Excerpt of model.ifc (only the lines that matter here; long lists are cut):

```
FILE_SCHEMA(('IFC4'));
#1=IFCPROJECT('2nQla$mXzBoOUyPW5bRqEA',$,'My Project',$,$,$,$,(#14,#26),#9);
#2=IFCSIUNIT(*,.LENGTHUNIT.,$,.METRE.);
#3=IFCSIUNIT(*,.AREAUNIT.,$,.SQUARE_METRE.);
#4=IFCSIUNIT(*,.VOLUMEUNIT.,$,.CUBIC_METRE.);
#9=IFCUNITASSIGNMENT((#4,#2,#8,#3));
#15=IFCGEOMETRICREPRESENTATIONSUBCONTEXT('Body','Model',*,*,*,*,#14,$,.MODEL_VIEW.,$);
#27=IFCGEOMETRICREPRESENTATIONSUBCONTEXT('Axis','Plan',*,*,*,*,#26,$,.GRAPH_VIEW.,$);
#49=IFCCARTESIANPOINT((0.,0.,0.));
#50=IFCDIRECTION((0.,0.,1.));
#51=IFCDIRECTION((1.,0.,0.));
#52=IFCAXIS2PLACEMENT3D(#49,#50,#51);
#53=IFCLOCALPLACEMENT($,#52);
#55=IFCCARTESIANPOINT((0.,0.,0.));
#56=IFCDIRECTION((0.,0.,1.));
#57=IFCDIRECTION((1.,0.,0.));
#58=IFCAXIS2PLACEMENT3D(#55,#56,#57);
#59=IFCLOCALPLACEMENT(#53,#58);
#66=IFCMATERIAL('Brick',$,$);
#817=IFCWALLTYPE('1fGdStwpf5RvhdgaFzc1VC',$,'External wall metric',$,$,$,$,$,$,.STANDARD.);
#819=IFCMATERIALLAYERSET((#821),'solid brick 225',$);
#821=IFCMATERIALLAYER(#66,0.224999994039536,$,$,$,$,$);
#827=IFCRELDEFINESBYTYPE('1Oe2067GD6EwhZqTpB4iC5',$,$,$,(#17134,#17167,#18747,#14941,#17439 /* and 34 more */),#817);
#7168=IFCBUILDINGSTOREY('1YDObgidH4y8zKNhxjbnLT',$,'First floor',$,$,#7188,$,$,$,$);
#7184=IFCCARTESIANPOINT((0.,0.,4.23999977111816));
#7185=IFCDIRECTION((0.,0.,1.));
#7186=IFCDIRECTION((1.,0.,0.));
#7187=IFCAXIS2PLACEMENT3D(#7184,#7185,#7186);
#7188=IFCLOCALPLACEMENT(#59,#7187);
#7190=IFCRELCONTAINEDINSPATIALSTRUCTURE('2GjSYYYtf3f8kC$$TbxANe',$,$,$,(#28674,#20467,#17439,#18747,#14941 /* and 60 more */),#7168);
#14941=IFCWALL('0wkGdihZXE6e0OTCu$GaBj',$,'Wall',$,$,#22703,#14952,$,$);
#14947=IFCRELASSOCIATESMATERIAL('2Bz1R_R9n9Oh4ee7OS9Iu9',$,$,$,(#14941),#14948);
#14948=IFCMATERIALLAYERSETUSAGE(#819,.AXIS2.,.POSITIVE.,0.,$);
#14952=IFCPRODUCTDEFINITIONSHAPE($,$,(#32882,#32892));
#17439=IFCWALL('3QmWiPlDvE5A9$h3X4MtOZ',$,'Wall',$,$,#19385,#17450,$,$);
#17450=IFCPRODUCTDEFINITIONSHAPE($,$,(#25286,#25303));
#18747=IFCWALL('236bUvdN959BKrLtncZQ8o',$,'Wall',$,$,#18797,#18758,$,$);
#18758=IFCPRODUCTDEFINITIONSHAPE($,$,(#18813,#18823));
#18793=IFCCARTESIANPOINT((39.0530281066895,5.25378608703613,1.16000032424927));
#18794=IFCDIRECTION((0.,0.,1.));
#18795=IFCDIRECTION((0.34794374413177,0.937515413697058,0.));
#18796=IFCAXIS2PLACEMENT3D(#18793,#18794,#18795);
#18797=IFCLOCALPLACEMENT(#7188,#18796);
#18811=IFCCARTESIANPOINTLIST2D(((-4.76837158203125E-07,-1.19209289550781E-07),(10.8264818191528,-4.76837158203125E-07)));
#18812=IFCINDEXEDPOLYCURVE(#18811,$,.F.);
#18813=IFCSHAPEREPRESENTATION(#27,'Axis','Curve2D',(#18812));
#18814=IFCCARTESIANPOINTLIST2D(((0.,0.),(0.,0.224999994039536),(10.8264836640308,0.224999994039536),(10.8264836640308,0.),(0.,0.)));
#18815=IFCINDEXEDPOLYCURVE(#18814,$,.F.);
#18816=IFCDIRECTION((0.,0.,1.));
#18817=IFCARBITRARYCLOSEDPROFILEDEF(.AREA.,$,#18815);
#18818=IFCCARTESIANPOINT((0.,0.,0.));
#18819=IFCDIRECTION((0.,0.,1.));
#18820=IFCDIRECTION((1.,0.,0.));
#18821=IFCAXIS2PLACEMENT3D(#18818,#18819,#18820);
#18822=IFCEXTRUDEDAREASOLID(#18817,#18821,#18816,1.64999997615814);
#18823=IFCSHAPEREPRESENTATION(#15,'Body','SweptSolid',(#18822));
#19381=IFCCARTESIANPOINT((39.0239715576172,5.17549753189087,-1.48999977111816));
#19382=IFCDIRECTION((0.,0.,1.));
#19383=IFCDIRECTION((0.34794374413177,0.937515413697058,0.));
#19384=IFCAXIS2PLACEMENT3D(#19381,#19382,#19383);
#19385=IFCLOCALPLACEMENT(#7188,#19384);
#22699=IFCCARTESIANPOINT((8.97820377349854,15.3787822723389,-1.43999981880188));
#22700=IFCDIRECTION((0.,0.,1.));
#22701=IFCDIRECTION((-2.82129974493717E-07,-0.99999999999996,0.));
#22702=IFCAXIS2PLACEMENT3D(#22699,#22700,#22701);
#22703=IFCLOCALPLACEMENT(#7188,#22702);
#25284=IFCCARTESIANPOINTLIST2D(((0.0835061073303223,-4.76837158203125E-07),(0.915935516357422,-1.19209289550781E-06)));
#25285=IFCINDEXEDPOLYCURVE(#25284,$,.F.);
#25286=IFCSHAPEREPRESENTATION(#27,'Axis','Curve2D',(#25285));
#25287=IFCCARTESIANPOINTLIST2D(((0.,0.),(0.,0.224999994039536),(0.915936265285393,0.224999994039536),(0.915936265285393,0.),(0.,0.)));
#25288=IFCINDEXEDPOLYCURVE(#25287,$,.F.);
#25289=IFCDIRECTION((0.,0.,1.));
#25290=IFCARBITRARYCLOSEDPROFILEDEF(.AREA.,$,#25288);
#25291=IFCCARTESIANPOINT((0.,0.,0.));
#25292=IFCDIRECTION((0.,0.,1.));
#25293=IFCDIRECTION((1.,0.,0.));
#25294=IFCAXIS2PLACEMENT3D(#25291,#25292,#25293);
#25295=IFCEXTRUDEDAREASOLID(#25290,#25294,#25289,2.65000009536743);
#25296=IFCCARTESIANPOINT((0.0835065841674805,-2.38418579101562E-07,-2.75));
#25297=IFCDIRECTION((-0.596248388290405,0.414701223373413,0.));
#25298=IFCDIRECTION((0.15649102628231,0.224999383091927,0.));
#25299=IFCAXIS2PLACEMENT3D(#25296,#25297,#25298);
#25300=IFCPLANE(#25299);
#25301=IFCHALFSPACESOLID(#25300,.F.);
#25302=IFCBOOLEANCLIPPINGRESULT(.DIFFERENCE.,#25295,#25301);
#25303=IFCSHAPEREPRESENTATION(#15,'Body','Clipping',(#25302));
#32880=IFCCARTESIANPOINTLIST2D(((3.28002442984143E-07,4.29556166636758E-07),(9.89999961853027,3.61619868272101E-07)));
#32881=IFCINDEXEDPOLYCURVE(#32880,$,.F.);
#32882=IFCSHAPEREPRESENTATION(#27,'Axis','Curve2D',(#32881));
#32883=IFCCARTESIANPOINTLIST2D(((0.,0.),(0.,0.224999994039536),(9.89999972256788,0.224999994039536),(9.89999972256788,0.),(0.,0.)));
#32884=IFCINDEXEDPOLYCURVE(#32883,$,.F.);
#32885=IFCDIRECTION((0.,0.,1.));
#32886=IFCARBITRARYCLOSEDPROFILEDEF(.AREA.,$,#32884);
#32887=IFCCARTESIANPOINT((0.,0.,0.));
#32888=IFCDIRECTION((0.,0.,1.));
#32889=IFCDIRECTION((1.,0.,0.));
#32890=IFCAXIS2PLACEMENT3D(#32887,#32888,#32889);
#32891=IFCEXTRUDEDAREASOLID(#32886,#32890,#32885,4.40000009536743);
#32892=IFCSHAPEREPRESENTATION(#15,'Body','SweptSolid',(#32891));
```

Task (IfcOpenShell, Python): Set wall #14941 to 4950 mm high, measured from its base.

```python
import ifcopenshell
import ifcopenshell.geom
import ifcopenshell.util.representation
import ifcopenshell.util.shape
import ifcopenshell.util.unit

model = ifcopenshell.open("model.ifc")
unit_scale = ifcopenshell.util.unit.calculate_unit_scale(model)
settings = ifcopenshell.geom.settings()


def volume(element):
    """Net volume in cubic metres, openings subtracted."""
    shape = ifcopenshell.geom.create_shape(settings, element)
    return ifcopenshell.util.shape.get_volume(shape.geometry)


wall = model.by_guid("0wkGdihZXE6e0OTCu$GaBj")
before = volume(wall)

body = ifcopenshell.util.representation.get_representation(wall, "Model", "Body")
solid = body.Items[0]
old_height = solid.Depth
solid.Depth = 4.95 / unit_scale
after = volume(wall)

print(f"height {old_height:g} -> {solid.Depth:g}, volume {before:.3f} -> {after:.3f} m3")

model.write("model_edited.ifc")
```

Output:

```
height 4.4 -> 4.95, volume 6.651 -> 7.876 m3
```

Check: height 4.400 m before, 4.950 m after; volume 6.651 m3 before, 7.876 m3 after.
